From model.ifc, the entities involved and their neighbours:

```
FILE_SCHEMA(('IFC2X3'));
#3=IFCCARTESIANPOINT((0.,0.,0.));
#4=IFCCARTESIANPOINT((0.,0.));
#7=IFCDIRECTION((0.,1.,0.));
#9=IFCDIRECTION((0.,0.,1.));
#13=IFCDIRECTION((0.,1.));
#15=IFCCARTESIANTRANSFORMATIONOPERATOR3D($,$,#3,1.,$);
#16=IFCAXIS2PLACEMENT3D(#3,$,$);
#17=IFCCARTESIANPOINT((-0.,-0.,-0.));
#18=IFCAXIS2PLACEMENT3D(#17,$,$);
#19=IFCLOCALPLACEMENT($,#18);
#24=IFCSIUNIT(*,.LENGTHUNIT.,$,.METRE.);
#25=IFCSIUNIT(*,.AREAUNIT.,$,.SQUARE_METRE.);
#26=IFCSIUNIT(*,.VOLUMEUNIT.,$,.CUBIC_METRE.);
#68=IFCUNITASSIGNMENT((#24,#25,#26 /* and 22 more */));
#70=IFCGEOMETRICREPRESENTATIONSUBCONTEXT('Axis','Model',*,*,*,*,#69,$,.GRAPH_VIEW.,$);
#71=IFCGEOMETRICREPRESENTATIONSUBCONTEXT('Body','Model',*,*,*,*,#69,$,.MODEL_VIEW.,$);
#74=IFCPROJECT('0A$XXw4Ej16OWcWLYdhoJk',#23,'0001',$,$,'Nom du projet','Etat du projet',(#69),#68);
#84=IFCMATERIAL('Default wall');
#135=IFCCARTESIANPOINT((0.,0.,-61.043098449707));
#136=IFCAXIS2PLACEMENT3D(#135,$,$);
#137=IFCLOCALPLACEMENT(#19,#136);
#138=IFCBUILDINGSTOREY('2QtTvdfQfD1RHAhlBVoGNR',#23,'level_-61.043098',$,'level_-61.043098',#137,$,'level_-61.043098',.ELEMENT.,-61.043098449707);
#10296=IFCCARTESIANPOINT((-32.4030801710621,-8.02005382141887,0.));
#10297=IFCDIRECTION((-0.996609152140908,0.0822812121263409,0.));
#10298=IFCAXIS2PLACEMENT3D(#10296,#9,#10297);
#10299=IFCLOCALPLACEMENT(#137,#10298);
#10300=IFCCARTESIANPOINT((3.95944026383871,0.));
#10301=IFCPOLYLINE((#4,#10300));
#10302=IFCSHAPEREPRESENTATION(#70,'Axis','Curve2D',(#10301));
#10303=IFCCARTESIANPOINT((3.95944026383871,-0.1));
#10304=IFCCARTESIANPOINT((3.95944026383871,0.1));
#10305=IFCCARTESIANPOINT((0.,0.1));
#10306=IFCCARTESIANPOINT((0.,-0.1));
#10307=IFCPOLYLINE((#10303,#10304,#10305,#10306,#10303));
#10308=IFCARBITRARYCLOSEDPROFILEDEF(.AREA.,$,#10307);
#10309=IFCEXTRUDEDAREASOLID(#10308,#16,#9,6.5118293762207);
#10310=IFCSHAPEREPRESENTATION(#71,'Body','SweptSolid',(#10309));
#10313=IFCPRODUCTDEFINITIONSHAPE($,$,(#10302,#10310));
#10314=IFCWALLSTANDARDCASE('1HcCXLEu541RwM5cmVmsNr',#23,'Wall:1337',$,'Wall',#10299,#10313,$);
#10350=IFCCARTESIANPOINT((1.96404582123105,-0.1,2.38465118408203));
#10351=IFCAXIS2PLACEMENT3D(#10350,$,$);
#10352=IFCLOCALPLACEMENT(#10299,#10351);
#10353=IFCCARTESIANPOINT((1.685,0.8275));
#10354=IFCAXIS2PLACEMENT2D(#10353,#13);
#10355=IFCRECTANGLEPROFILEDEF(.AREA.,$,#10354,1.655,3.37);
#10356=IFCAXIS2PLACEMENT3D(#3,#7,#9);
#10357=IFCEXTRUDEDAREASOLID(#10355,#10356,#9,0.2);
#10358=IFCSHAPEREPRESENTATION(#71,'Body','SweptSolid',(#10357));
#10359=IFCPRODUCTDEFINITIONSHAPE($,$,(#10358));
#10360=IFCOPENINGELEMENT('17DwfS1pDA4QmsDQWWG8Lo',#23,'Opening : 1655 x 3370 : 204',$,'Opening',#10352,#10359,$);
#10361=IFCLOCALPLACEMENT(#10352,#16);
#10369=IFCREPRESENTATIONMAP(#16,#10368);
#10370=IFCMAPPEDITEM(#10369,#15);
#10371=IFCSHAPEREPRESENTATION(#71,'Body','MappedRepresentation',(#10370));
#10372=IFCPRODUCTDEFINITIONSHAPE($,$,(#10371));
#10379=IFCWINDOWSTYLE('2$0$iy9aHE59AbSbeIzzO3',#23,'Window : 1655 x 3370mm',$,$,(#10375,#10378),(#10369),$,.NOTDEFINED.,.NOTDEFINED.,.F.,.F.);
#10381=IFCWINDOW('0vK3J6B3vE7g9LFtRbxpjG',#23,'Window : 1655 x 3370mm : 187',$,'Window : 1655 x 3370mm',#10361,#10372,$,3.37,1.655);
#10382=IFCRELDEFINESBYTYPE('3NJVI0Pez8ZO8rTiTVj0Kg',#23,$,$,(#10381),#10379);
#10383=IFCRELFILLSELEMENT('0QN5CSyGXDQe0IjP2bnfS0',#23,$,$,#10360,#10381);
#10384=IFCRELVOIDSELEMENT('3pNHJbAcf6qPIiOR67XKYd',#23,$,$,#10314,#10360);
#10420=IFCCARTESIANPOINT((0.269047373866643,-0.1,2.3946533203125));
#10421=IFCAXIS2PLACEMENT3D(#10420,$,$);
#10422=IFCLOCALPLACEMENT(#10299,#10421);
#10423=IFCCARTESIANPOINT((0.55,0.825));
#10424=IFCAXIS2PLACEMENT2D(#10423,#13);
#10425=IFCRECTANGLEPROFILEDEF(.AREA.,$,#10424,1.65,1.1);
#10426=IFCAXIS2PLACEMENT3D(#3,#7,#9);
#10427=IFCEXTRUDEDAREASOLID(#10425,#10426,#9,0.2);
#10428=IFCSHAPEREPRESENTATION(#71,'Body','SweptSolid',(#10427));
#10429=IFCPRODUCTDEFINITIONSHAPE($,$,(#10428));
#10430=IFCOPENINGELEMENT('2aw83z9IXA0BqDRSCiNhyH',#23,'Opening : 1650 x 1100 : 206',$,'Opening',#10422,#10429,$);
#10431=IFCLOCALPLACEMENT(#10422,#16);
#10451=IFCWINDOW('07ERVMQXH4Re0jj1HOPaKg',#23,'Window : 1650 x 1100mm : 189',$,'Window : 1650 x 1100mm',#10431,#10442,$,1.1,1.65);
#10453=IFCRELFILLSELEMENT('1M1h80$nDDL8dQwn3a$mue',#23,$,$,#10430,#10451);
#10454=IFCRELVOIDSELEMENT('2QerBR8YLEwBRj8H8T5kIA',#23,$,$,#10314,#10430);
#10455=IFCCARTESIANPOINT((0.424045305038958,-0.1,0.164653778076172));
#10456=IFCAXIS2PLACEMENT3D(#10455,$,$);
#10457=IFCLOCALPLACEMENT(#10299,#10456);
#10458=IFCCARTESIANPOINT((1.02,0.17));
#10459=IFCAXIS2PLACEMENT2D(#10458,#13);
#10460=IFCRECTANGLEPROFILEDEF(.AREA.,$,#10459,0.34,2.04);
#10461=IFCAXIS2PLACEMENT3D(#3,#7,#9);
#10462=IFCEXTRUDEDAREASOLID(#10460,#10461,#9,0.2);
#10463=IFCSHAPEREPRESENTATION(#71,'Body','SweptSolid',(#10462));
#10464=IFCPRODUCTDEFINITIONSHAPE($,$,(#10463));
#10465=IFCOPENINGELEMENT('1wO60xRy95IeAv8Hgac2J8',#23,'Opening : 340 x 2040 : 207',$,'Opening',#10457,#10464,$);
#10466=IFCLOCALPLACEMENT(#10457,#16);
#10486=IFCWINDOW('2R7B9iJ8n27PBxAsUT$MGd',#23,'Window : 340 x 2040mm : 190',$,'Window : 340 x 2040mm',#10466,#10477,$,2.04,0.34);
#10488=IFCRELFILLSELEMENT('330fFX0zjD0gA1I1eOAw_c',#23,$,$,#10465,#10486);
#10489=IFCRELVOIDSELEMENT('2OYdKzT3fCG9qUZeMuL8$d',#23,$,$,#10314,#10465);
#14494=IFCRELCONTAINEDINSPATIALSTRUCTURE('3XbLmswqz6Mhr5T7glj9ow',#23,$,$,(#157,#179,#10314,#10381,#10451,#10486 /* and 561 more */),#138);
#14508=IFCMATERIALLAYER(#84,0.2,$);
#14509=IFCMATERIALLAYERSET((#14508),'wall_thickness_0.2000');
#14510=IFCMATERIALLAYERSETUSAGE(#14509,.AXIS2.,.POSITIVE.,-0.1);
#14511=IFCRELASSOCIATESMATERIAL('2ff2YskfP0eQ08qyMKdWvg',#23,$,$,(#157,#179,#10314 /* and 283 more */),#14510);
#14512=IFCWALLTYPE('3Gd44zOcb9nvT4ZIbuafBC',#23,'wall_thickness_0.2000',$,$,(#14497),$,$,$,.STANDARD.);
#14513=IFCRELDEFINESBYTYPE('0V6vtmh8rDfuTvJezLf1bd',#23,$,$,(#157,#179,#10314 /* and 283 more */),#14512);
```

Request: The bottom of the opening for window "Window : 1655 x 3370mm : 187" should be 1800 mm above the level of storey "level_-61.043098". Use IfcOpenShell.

```python
import numpy as np
import ifcopenshell
import ifcopenshell.api.geometry
import ifcopenshell.geom
import ifcopenshell.util.element
import ifcopenshell.util.placement
import ifcopenshell.util.shape
import ifcopenshell.util.unit

model = ifcopenshell.open("model.ifc")
unit_scale = ifcopenshell.util.unit.calculate_unit_scale(model)

window = model.by_guid("0vK3J6B3vE7g9LFtRbxpjG")
opening = window.FillsVoids[0].RelatingOpeningElement
storey = ifcopenshell.util.element.get_container(window, ifc_class="IfcBuildingStorey")
level = ifcopenshell.util.placement.get_local_placement(storey.ObjectPlacement)[2, 3]

# The opening's origin need not be at the sill, so measure its lowest point.
shape = ifcopenshell.geom.create_shape(ifcopenshell.geom.settings(), opening)
bottom = ifcopenshell.util.shape.get_shape_bottom_elevation(shape, shape.geometry) / unit_scale
dz = level + 1.8 / unit_scale - bottom

shift = np.array([0.0, 0.0, dz])
# The window is placed relative to its opening, so it follows when the opening moves.
matrix = ifcopenshell.util.placement.get_local_placement(opening.ObjectPlacement)
matrix[:3, 3] += shift
ifcopenshell.api.geometry.edit_object_placement(
    model, product=opening, matrix=matrix, is_si=False, should_transform_children=True
)

print(f"moved by {dz * unit_scale:+.3f} m")

model.write("model-out.ifc")
```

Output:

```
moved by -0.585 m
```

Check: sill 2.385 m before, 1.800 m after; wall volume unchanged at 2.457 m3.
